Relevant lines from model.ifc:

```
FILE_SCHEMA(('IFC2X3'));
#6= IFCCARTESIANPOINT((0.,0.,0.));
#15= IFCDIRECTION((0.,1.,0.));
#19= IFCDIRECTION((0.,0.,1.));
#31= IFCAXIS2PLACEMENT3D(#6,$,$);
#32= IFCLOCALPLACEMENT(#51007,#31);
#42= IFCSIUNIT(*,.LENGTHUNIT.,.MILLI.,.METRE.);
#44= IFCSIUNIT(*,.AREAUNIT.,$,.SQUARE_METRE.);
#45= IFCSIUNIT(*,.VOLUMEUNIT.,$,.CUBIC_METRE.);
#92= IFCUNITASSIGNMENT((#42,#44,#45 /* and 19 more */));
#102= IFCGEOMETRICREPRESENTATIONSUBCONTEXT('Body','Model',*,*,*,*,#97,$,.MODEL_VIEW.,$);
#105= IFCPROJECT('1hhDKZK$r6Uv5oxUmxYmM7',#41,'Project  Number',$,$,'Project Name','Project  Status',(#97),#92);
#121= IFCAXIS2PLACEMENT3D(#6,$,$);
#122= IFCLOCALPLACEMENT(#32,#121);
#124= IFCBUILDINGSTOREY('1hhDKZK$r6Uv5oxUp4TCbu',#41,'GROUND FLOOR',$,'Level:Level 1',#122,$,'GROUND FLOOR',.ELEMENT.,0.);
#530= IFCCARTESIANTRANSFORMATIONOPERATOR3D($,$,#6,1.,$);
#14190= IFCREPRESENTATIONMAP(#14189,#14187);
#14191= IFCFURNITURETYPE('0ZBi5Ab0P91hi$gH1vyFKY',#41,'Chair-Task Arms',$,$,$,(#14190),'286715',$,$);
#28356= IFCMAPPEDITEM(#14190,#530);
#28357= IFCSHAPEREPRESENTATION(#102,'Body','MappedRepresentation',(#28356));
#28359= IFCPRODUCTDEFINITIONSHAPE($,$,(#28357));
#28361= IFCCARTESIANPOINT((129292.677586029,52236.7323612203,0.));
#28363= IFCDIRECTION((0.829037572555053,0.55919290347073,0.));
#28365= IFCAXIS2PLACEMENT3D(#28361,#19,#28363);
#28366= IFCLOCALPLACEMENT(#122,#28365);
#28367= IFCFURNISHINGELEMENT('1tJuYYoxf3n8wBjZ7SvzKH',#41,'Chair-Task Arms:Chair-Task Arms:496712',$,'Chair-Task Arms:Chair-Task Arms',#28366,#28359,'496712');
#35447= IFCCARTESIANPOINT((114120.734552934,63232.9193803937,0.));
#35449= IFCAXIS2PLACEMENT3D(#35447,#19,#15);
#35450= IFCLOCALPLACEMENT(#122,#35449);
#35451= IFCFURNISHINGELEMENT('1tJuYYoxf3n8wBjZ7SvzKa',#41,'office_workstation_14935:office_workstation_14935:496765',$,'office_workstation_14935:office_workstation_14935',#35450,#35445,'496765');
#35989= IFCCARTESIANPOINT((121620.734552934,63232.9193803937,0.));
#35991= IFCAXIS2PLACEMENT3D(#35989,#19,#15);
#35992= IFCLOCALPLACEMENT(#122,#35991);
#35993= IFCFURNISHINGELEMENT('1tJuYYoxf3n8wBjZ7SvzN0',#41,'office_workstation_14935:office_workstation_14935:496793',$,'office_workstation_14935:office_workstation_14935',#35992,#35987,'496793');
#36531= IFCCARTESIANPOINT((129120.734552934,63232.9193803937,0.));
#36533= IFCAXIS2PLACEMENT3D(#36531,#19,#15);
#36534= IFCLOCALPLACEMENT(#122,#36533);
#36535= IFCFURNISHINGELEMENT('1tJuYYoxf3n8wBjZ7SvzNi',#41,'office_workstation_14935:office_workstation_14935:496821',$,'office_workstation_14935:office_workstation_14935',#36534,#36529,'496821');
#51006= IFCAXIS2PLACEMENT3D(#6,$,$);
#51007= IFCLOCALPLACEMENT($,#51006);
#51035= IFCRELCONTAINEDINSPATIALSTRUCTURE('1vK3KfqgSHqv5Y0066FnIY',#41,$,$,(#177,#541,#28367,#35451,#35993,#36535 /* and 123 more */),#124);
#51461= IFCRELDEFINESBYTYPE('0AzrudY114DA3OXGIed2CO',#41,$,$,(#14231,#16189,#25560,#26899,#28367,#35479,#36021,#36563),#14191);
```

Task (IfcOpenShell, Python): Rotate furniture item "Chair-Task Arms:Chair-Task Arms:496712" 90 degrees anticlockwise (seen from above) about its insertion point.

```python
import ifcopenshell
import ifcopenshell.api.geometry
import ifcopenshell.util.placement

model = ifcopenshell.open("model.ifc")

item = model.by_guid("1tJuYYoxf3n8wBjZ7SvzKH")
matrix = ifcopenshell.util.placement.get_local_placement(item.ObjectPlacement)
matrix = matrix @ ifcopenshell.util.placement.rotation(90, "Z")
ifcopenshell.api.geometry.edit_object_placement(model, product=item, matrix=matrix, is_si=False)

print(ifcopenshell.util.placement.get_local_placement(item.ObjectPlacement).round(3) + 0.0)

model.write("model_updated.ifc")
```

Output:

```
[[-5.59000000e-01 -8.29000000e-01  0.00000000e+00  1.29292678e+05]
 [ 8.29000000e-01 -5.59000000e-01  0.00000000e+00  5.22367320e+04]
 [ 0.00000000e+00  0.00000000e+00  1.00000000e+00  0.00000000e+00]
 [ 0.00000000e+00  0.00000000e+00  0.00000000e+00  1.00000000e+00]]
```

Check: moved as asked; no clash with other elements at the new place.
